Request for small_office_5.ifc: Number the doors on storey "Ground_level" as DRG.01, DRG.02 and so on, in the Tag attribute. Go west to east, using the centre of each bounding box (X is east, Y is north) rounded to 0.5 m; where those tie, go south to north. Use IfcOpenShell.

First a look at what the model holds.

```python
import ifcopenshell
import ifcopenshell.util.element
import ifcopenshell.util.placement

model = ifcopenshell.open("small_office_5.ifc")
print(model.schema)
storey = next(s for s in model.by_type("IfcBuildingStorey") if s.Name == "Ground_level")
doors = [e for e in ifcopenshell.util.element.get_decomposition(storey) if e.is_a("IfcDoor")]
for e in sorted(doors, key=lambda e: e.id()):
    origin = ifcopenshell.util.placement.get_local_placement(e.ObjectPlacement)[:3, 3]
    print(e.id(), e.Tag, e.Name, origin.round(2) + 0.0, sep=" | ")
```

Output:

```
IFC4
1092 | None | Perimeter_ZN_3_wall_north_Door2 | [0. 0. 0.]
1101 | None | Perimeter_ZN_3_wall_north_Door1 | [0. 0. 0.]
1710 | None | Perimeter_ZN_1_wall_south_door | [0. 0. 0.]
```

```python
import ifcopenshell
import ifcopenshell.geom
import ifcopenshell.util.element
import ifcopenshell.util.shape

model = ifcopenshell.open("small_office_5.ifc")
settings = ifcopenshell.geom.settings()
settings.set("use-world-coords", True)


def centre(element):
    shape = ifcopenshell.geom.create_shape(settings, element)
    return ifcopenshell.util.shape.get_bbox_centroid(shape.geometry)


storey = next(s for s in model.by_type("IfcBuildingStorey") if s.Name == "Ground_level")
doors = [e for e in ifcopenshell.util.element.get_decomposition(storey) if e.is_a("IfcDoor")]

# Insertion points can sit at a corner or the storey origin, so sort by the geometry (in metres).
centres = {e: centre(e) for e in doors}
doors.sort(key=lambda e: (round(centres[e][0] / 0.5), centres[e][1]))

for i, e in enumerate(doors, start=1):
    number = f"DRG.{i:02d}"
    e.Tag = number
    print(e.id(), number)

model.write("small_office_5_v2.ifc")
```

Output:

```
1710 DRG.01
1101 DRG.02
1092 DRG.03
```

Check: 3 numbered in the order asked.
